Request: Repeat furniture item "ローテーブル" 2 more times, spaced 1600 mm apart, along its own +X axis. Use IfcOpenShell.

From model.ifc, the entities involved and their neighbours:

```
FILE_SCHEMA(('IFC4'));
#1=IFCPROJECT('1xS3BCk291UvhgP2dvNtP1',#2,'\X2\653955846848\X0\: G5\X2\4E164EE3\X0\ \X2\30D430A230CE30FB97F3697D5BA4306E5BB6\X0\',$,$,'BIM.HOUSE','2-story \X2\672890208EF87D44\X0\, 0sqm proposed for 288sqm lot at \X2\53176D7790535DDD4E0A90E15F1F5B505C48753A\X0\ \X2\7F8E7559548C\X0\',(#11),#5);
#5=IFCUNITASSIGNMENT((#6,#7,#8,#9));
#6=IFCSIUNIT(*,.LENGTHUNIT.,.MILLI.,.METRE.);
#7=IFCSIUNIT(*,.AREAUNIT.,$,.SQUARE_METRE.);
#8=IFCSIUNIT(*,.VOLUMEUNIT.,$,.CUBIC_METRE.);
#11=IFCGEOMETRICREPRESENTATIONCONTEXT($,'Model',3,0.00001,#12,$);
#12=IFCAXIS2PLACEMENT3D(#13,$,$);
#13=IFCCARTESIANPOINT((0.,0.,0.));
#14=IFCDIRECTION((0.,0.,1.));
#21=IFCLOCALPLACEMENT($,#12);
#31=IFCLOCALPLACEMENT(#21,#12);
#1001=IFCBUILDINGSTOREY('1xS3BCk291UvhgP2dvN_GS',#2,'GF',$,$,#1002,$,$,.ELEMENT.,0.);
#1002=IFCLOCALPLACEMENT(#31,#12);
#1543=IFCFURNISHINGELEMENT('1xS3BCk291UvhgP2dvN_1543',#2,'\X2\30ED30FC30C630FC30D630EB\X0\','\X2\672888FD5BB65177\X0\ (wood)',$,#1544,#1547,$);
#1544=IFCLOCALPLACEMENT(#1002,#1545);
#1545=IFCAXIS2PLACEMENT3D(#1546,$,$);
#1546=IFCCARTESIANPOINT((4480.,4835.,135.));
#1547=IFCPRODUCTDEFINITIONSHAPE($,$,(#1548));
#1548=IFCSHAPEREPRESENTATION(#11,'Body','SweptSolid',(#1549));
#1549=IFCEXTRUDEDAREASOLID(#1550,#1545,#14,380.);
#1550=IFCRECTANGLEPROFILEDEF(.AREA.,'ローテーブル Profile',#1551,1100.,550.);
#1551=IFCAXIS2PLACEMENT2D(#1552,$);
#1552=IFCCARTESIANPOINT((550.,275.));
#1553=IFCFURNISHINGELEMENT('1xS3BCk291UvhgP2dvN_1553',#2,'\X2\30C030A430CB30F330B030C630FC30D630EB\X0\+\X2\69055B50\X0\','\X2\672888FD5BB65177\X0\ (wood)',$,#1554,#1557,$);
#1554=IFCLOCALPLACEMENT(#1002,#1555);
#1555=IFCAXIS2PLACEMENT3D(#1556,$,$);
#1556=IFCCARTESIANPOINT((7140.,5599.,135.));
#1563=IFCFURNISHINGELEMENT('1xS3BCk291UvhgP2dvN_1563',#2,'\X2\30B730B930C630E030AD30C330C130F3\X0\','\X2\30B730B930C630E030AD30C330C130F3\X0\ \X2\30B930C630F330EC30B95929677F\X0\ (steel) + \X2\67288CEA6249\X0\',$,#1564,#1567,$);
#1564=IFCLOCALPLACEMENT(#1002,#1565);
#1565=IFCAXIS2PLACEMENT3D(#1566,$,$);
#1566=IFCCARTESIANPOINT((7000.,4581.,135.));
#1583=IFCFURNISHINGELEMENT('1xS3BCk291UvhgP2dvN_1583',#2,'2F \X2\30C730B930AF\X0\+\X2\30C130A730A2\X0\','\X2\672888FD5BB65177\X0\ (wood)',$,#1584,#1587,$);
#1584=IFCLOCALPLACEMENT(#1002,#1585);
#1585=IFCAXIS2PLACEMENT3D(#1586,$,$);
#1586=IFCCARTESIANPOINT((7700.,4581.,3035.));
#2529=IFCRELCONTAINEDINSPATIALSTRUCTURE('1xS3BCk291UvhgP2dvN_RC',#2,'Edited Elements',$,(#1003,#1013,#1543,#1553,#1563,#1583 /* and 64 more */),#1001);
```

```python
import ifcopenshell
import ifcopenshell.api.geometry
import ifcopenshell.api.root
import ifcopenshell.util.element
import ifcopenshell.util.placement
import ifcopenshell.util.unit

model = ifcopenshell.open("model.ifc")
unit_scale = ifcopenshell.util.unit.calculate_unit_scale(model)


def reuse_history(source, copy):
    """copy_class also copies each property set's owner history, people and application; keep the originals."""
    for rel in copy.IsDefinedBy:
        if rel.is_a("IfcRelDefinesByProperties") and (history := rel.RelatingPropertyDefinition.OwnerHistory):
            rel.RelatingPropertyDefinition.OwnerHistory = source.OwnerHistory
            ifcopenshell.util.element.remove_deep2(model, history)


source = model.by_guid("1xS3BCk291UvhgP2dvN_1543")
base = ifcopenshell.util.placement.get_local_placement(source.ObjectPlacement)
step = base[:3, 0] * 1.6 / unit_scale

for i in range(1, 3):
    copy = ifcopenshell.api.root.copy_class(model, product=source)
    copy.Representation = ifcopenshell.util.element.copy_deep(
        model, source.Representation, exclude=["IfcGeometricRepresentationContext", "IfcRepresentationMap"]
    )
    reuse_history(source, copy)
    matrix = base.copy()
    matrix[:3, 3] += i * step
    print("added at", matrix[:3, 3].round(3) + 0.0)
    ifcopenshell.api.geometry.edit_object_placement(model, product=copy, matrix=matrix, is_si=False)

model.write("model-out.ifc")
```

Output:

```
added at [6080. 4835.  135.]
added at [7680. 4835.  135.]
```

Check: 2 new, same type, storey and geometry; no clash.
